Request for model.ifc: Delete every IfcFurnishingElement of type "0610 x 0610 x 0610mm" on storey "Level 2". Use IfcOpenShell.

First a look at what the model holds.

```python
import ifcopenshell
import ifcopenshell.util.element

model = ifcopenshell.open("model.ifc")
print(model.schema)
storey = next(s for s in model.by_type("IfcBuildingStorey") if s.Name == "Level 2")
furniture = [e for e in ifcopenshell.util.element.get_decomposition(storey) if e.is_a("IfcFurnishingElement")]
seen = {}
for e in furniture:
    element_type = ifcopenshell.util.element.get_type(e)
    name = element_type.Name if element_type not in (None, e) else None
    seen[name] = seen.get(name, 0) + 1
for name, count in sorted(seen.items(), key=str):
    print(count, "x", name)
```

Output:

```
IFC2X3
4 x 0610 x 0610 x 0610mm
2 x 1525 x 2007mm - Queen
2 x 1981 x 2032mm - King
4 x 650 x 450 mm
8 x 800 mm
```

```python
import ifcopenshell
import ifcopenshell.api.root
import ifcopenshell.util.element

model = ifcopenshell.open("model.ifc")

storey = next(s for s in model.by_type("IfcBuildingStorey") if s.Name == "Level 2")
furniture = [e for e in ifcopenshell.util.element.get_decomposition(storey) if e.is_a("IfcFurnishingElement")]
targets = [e for e in furniture if (t := ifcopenshell.util.element.get_type(e)) not in (None, e) and t.Name == "0610 x 0610 x 0610mm"]

for e in targets:
    ifcopenshell.api.root.remove_product(model, product=e)
print(len(targets), "removed")

model.write("model_v2.ifc")
```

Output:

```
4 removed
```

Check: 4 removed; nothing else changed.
